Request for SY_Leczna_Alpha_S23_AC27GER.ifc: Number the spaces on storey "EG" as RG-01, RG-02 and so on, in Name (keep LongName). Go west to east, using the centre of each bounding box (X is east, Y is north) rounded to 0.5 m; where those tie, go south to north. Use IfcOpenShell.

First a look at what the model holds.

```python
import ifcopenshell
import ifcopenshell.util.element
import ifcopenshell.util.placement

model = ifcopenshell.open("SY_Leczna_Alpha_S23_AC27GER.ifc")
print(model.schema)
storey = next(s for s in model.by_type("IfcBuildingStorey") if s.Name == "EG")
spaces = [e for e in ifcopenshell.util.element.get_decomposition(storey) if e.is_a("IfcSpace")]
for e in sorted(spaces, key=lambda e: e.id()):
    origin = ifcopenshell.util.placement.get_local_placement(e.ObjectPlacement)[:3, 3]
    print(e.id(), e.Name, e.LongName, origin.round(2) + 0.0, sep=" | ")
```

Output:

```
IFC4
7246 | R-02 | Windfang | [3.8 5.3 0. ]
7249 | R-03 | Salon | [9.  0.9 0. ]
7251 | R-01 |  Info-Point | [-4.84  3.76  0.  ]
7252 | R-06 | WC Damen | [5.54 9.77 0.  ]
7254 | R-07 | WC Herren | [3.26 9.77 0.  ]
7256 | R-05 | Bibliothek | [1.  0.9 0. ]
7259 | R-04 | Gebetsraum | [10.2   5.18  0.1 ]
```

```python
import ifcopenshell
import ifcopenshell.geom
import ifcopenshell.util.element
import ifcopenshell.util.shape

model = ifcopenshell.open("SY_Leczna_Alpha_S23_AC27GER.ifc")
settings = ifcopenshell.geom.settings()
settings.set("use-world-coords", True)


def centre(element):
    shape = ifcopenshell.geom.create_shape(settings, element)
    return ifcopenshell.util.shape.get_bbox_centroid(shape.geometry)


storey = next(s for s in model.by_type("IfcBuildingStorey") if s.Name == "EG")
spaces = [e for e in ifcopenshell.util.element.get_decomposition(storey) if e.is_a("IfcSpace")]

# Insertion points can sit at a corner or the storey origin, so sort by the geometry (in metres).
centres = {e: centre(e) for e in spaces}
spaces.sort(key=lambda e: (round(centres[e][0] / 0.5), centres[e][1]))

for i, e in enumerate(spaces, start=1):
    number = f"RG-{i:02d}"
    e.Name = number
    print(e.id(), number)

model.write("SY_Leczna_Alpha_S23_AC27GER_v2.ifc")
```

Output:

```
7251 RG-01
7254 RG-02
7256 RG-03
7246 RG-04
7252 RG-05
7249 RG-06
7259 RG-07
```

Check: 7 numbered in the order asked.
